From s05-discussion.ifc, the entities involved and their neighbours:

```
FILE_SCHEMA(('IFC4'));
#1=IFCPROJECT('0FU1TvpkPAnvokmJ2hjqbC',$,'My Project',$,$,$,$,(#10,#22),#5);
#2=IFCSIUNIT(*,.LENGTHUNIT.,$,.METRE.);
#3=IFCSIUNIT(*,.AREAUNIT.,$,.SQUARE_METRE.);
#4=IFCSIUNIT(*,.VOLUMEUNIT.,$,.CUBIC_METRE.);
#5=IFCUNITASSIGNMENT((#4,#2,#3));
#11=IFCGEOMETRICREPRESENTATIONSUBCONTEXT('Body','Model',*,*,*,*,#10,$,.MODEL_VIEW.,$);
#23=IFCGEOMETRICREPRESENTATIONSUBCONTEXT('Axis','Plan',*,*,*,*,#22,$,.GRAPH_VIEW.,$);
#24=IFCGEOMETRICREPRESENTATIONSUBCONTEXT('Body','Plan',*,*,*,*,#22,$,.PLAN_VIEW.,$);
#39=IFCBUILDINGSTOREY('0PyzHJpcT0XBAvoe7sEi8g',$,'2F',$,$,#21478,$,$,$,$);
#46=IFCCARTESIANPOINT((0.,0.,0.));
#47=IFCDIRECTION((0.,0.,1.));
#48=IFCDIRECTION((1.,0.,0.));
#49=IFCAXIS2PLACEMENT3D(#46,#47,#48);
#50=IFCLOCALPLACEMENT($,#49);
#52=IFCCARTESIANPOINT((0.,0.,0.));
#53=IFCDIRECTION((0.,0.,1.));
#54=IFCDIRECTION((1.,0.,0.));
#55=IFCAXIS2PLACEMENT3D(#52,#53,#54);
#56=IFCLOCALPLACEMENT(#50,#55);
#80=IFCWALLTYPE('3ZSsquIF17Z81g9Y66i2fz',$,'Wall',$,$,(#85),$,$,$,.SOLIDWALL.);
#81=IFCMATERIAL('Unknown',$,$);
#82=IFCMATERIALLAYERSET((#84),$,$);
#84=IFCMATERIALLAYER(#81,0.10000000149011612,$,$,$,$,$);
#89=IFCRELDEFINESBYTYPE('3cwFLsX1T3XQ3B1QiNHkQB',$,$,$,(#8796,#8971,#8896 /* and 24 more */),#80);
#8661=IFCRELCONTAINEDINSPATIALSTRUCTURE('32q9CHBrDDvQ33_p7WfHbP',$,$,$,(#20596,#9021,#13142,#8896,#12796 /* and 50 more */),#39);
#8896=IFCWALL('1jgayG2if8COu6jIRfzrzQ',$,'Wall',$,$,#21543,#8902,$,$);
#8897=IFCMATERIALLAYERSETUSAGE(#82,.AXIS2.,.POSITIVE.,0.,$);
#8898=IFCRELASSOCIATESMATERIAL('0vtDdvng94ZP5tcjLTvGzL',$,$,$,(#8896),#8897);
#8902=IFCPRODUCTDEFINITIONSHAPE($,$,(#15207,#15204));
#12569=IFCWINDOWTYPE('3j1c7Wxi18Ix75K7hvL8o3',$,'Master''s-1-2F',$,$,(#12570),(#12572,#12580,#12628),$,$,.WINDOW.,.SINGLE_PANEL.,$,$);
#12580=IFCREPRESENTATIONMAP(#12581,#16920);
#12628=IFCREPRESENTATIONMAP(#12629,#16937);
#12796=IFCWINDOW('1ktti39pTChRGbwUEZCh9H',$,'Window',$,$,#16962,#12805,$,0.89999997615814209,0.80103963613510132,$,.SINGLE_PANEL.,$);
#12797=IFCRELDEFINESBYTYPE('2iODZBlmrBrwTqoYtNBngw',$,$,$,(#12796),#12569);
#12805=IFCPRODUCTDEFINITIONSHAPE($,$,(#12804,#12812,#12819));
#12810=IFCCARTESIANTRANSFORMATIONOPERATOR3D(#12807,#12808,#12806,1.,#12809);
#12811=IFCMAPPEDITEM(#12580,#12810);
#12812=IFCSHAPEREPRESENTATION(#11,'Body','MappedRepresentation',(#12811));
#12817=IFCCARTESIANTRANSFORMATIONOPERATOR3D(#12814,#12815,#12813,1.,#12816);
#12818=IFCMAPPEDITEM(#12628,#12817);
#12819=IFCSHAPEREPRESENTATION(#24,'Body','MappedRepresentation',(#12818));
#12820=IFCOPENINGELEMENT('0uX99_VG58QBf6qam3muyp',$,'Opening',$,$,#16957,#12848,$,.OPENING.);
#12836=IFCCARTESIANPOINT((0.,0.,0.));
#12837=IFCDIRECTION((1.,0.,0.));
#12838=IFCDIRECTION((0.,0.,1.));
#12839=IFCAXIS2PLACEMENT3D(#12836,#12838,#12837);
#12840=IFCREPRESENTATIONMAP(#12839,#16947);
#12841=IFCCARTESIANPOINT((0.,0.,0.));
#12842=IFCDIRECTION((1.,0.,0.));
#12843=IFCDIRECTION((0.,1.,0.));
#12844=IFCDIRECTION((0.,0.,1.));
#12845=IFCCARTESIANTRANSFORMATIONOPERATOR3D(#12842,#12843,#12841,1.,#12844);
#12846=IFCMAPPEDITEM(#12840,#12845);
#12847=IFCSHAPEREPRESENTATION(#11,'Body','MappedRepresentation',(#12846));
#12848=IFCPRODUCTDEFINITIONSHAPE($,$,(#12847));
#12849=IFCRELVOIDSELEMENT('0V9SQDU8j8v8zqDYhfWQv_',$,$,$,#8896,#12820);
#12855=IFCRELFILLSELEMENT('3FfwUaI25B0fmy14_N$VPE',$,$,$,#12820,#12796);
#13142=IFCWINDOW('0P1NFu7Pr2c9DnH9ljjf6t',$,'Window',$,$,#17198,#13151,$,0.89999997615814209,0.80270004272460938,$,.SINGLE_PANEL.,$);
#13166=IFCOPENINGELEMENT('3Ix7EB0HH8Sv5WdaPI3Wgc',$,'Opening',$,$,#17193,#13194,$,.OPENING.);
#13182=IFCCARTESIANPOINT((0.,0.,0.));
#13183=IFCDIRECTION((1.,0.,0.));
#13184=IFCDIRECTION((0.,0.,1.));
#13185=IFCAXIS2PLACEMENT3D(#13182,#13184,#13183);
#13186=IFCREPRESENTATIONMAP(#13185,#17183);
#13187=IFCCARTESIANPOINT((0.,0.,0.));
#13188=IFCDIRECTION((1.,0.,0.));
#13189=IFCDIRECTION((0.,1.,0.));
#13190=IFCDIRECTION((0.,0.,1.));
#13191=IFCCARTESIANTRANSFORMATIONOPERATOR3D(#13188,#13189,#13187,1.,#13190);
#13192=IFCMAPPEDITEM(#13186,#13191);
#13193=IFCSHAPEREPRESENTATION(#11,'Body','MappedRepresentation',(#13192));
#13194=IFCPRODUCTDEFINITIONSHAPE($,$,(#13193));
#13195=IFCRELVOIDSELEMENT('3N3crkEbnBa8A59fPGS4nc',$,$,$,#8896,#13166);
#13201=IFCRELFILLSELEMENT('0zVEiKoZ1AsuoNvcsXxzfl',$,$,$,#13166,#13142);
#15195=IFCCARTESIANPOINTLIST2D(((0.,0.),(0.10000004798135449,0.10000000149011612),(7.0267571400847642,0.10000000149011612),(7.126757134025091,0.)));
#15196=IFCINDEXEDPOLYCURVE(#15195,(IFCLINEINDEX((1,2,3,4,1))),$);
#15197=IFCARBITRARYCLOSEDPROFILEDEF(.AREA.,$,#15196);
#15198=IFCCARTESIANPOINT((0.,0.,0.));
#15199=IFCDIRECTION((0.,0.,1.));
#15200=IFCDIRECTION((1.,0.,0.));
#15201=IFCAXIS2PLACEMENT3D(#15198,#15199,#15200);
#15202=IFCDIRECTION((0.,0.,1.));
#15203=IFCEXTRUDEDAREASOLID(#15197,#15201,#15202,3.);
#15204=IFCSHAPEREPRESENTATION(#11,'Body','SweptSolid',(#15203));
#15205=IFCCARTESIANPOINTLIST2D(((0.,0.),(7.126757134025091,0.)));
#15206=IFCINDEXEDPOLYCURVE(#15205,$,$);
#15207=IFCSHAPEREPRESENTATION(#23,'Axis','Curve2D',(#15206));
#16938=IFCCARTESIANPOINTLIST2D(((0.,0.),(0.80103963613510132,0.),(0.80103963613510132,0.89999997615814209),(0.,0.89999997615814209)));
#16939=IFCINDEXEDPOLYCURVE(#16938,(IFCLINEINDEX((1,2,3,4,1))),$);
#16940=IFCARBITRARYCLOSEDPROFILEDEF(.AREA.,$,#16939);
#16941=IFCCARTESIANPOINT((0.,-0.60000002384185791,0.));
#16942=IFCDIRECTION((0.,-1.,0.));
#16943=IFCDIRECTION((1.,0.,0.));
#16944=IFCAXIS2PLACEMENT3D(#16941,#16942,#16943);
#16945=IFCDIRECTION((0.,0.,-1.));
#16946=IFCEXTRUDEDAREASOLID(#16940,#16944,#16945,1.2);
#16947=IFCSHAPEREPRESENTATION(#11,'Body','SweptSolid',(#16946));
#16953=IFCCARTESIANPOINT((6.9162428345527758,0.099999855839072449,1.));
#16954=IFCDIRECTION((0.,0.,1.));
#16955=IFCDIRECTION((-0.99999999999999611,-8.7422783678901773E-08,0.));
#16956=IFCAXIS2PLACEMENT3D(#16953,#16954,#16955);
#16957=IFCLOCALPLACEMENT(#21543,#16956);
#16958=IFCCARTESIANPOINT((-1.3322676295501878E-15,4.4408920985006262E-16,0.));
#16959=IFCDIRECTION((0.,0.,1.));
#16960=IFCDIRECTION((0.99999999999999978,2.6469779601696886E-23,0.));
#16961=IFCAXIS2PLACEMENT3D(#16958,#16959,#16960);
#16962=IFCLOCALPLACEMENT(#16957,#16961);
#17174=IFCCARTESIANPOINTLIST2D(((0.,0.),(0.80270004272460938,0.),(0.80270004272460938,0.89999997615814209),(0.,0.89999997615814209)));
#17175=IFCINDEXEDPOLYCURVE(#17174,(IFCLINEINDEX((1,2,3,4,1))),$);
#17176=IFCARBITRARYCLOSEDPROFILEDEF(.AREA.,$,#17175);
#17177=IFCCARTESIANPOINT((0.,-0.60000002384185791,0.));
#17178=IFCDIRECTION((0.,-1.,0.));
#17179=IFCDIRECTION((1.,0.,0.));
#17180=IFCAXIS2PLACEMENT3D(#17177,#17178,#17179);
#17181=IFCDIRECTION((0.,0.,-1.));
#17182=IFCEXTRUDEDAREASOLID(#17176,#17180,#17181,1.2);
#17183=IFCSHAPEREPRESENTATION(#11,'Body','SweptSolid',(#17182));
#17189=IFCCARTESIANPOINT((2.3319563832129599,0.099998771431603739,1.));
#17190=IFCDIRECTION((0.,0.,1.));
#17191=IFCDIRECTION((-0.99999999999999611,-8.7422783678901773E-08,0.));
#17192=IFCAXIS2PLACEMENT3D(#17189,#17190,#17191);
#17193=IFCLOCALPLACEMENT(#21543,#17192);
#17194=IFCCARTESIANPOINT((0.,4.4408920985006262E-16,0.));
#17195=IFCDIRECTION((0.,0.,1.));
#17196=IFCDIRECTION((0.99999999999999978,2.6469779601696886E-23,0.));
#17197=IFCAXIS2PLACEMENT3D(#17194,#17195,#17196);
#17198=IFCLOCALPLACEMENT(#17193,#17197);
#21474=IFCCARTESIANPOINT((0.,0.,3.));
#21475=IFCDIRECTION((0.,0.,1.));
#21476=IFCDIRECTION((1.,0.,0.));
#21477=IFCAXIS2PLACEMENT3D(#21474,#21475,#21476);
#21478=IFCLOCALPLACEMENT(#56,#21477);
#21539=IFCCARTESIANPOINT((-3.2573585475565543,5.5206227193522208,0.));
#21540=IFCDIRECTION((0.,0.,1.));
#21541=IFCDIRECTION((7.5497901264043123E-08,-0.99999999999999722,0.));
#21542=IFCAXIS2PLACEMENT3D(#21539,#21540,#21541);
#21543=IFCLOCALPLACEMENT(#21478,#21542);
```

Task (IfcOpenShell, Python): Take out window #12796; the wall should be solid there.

```python
import ifcopenshell
import ifcopenshell.api.feature
import ifcopenshell.api.root
import ifcopenshell.geom
import ifcopenshell.util.shape

model = ifcopenshell.open("s05-discussion.ifc")
settings = ifcopenshell.geom.settings()


def volume(element):
    """Net volume in cubic metres, openings subtracted."""
    shape = ifcopenshell.geom.create_shape(settings, element)
    return ifcopenshell.util.shape.get_volume(shape.geometry)


window = model.by_guid("1ktti39pTChRGbwUEZCh9H")
opening = window.FillsVoids[0].RelatingOpeningElement
wall = opening.VoidsElements[0].RelatingBuildingElement
before = volume(wall)

ifcopenshell.api.root.remove_product(model, product=window)
ifcopenshell.api.feature.remove_feature(model, feature=opening)

after = volume(wall)

print(f"wall volume {before:.3f} -> {after:.3f} m3")

model.write("s05-discussion_updated.ifc")
```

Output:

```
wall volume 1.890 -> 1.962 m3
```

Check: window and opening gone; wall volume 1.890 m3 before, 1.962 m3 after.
